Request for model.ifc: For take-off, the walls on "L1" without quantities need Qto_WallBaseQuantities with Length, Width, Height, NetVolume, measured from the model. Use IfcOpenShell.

First a look at what the model holds.

```python
import ifcopenshell
import ifcopenshell.util.element
import ifcopenshell.util.unit

model = ifcopenshell.open("model.ifc")
print(model.schema)
for unit_type in ("LENGTHUNIT", "AREAUNIT", "VOLUMEUNIT"):
    print(unit_type, ifcopenshell.util.unit.calculate_unit_scale(model, unit_type))
storey = next(s for s in model.by_type("IfcBuildingStorey") if s.Name == "L1")
walls = [e for e in ifcopenshell.util.element.get_decomposition(storey) if e.is_a("IfcWall")]
for e in sorted(walls, key=lambda e: e.id()):
    print(e.id(), e.is_a(), e.Name, list(ifcopenshell.util.element.get_psets(e, qtos_only=True)), sep=" | ")
```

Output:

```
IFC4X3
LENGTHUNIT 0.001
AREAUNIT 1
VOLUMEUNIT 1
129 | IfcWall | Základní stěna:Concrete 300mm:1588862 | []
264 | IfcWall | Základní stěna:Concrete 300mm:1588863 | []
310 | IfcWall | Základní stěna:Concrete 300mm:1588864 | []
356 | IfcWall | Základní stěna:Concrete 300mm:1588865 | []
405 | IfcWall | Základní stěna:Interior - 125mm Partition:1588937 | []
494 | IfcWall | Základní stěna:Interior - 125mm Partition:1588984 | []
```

```python
import ifcopenshell
import ifcopenshell.api.pset
import ifcopenshell.geom
import ifcopenshell.util.element
import ifcopenshell.util.shape
import ifcopenshell.util.unit

model = ifcopenshell.open("model.ifc")
unit_scale = ifcopenshell.util.unit.calculate_unit_scale(model)
volume_scale = ifcopenshell.util.unit.calculate_unit_scale(model, "VOLUMEUNIT")
settings = ifcopenshell.geom.settings()

storey = next(s for s in model.by_type("IfcBuildingStorey") if s.Name == "L1")
walls = [e for e in ifcopenshell.util.element.get_decomposition(storey) if e.is_a("IfcWall")]

for e in sorted(walls, key=lambda e: e.id()):
    if ifcopenshell.util.element.get_psets(e, qtos_only=True, should_inherit=False):
        continue
    # Geometry comes back in metres, in the element's own axes.
    shape = ifcopenshell.geom.create_shape(settings, e)
    values = {
        "Length": ifcopenshell.util.shape.get_x(shape.geometry) / unit_scale,
        "Width": ifcopenshell.util.shape.get_y(shape.geometry) / unit_scale,
        "Height": ifcopenshell.util.shape.get_z(shape.geometry) / unit_scale,
        "NetVolume": ifcopenshell.util.shape.get_volume(shape.geometry) / volume_scale,
    }
    qto = ifcopenshell.api.pset.add_qto(model, product=e, name="Qto_WallBaseQuantities")
    ifcopenshell.api.pset.edit_qto(model, qto=qto, properties=values)
    print(e.id(), {k: round(v, 3) for k, v in values.items()})

model.write("model_rev.ifc")
```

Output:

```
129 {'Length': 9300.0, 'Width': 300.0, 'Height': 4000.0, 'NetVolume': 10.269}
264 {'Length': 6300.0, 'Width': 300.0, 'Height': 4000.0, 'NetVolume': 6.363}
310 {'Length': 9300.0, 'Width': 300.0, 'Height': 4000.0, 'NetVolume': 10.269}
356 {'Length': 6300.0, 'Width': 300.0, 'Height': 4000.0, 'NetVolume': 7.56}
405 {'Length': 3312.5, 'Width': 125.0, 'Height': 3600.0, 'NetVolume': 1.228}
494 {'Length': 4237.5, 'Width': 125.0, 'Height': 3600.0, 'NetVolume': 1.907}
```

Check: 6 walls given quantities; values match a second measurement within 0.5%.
